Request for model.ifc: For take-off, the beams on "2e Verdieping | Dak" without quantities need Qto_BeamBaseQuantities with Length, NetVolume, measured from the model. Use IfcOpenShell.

First a look at what the model holds.

```python
import ifcopenshell
import ifcopenshell.util.element
import ifcopenshell.util.unit

model = ifcopenshell.open("model.ifc")
print(model.schema)
for unit_type in ("LENGTHUNIT", "AREAUNIT", "VOLUMEUNIT"):
    print(unit_type, ifcopenshell.util.unit.calculate_unit_scale(model, unit_type))
storey = next(s for s in model.by_type("IfcBuildingStorey") if s.Name == "2e Verdieping | Dak")
beams = [e for e in ifcopenshell.util.element.get_decomposition(storey) if e.is_a("IfcBeam")]
for e in sorted(beams, key=lambda e: e.id()):
    print(e.id(), e.is_a(), e.Name, list(ifcopenshell.util.element.get_psets(e, qtos_only=True)), sep=" | ")
```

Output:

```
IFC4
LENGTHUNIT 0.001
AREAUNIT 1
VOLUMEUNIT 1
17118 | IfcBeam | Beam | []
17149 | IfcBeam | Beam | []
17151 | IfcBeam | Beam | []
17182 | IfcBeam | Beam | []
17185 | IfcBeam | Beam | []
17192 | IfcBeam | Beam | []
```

```python
import ifcopenshell
import ifcopenshell.api.pset
import ifcopenshell.geom
import ifcopenshell.util.element
import ifcopenshell.util.shape
import ifcopenshell.util.unit

model = ifcopenshell.open("model.ifc")
unit_scale = ifcopenshell.util.unit.calculate_unit_scale(model)
volume_scale = ifcopenshell.util.unit.calculate_unit_scale(model, "VOLUMEUNIT")
settings = ifcopenshell.geom.settings()

storey = next(s for s in model.by_type("IfcBuildingStorey") if s.Name == "2e Verdieping | Dak")
beams = [e for e in ifcopenshell.util.element.get_decomposition(storey) if e.is_a("IfcBeam")]

for e in sorted(beams, key=lambda e: e.id()):
    if ifcopenshell.util.element.get_psets(e, qtos_only=True, should_inherit=False):
        continue
    # Geometry comes back in metres, in the element's own axes.
    shape = ifcopenshell.geom.create_shape(settings, e)
    values = {
        "Length": ifcopenshell.util.shape.get_max_xyz(shape.geometry) / unit_scale,
        "NetVolume": ifcopenshell.util.shape.get_volume(shape.geometry) / volume_scale,
    }
    qto = ifcopenshell.api.pset.add_qto(model, product=e, name="Qto_BeamBaseQuantities")
    ifcopenshell.api.pset.edit_qto(model, qto=qto, properties=values)
    print(e.id(), {k: round(v, 3) for k, v in values.items()})

model.write("model_edited.ifc")
```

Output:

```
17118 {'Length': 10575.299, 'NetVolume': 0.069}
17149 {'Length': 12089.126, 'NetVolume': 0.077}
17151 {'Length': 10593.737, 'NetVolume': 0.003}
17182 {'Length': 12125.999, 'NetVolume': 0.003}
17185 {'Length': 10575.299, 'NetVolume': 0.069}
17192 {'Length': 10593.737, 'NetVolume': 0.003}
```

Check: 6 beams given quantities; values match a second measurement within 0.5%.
